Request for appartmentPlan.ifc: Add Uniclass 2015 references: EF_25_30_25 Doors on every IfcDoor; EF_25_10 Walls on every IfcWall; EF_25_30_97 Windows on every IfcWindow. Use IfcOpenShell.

First a look at what the model holds.

```python
import ifcopenshell

model = ifcopenshell.open("appartmentPlan.ifc")
print(model.schema)
print("classifications:", [c.Name for c in model.by_type("IfcClassification")])
for ifc_class in ("IfcDoor", "IfcRoof", "IfcStair", "IfcWall", "IfcWindow"):
    print(ifc_class, len(model.by_type(ifc_class)))
```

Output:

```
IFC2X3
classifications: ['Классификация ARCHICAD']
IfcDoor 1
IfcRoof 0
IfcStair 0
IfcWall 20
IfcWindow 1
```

```python
import ifcopenshell
import ifcopenshell.api.classification

model = ifcopenshell.open("appartmentPlan.ifc")

# IFC2X3 requires Source and Edition and has no link from the project to the system.
system = model.create_entity("IfcClassification", Source="NBS", Edition="2015", Name="Uniclass 2015")

codes = {
    "IfcDoor": ("EF_25_30_25", "Doors"),
    "IfcWall": ("EF_25_10", "Walls"),
    "IfcWindow": ("EF_25_30_97", "Windows"),
}
for ifc_class, (code, name) in codes.items():
    products = model.by_type(ifc_class)
    ifcopenshell.api.classification.add_reference(
        model, products=products, classification=system, identification=code, name=name
    )
    print(code, len(products))

model.write("appartmentPlan_updated.ifc")
```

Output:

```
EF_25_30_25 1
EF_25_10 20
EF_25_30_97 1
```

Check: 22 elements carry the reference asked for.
